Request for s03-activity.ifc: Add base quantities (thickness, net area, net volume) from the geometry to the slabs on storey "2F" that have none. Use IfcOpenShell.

First a look at what the model holds.

```python
import ifcopenshell
import ifcopenshell.util.element
import ifcopenshell.util.unit

model = ifcopenshell.open("s03-activity.ifc")
print(model.schema)
for unit_type in ("LENGTHUNIT", "AREAUNIT", "VOLUMEUNIT"):
    print(unit_type, ifcopenshell.util.unit.calculate_unit_scale(model, unit_type))
storey = next(s for s in model.by_type("IfcBuildingStorey") if s.Name == "2F")
slabs = [e for e in ifcopenshell.util.element.get_decomposition(storey) if e.is_a("IfcSlab")]
for e in sorted(slabs, key=lambda e: e.id()):
    print(e.id(), e.is_a(), e.Name, list(ifcopenshell.util.element.get_psets(e, qtos_only=True)), sep=" | ")
```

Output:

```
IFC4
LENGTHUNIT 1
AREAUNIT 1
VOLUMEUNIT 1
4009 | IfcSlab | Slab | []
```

```python
import ifcopenshell
import ifcopenshell.api.pset
import ifcopenshell.geom
import ifcopenshell.util.element
import ifcopenshell.util.shape
import ifcopenshell.util.unit

model = ifcopenshell.open("s03-activity.ifc")
unit_scale = ifcopenshell.util.unit.calculate_unit_scale(model)
area_scale = ifcopenshell.util.unit.calculate_unit_scale(model, "AREAUNIT")
volume_scale = ifcopenshell.util.unit.calculate_unit_scale(model, "VOLUMEUNIT")
settings = ifcopenshell.geom.settings()

storey = next(s for s in model.by_type("IfcBuildingStorey") if s.Name == "2F")
slabs = [e for e in ifcopenshell.util.element.get_decomposition(storey) if e.is_a("IfcSlab")]

for e in sorted(slabs, key=lambda e: e.id()):
    if ifcopenshell.util.element.get_psets(e, qtos_only=True, should_inherit=False):
        continue
    # Geometry comes back in metres, in the element's own axes.
    shape = ifcopenshell.geom.create_shape(settings, e)
    values = {
        "Width": ifcopenshell.util.shape.get_z(shape.geometry) / unit_scale,
        "NetArea": ifcopenshell.util.shape.get_footprint_area(shape.geometry) / area_scale,
        "NetVolume": ifcopenshell.util.shape.get_volume(shape.geometry) / volume_scale,
    }
    qto = ifcopenshell.api.pset.add_qto(model, product=e, name="Qto_SlabBaseQuantities")
    ifcopenshell.api.pset.edit_qto(model, qto=qto, properties=values)
    print(e.id(), {k: round(v, 3) for k, v in values.items()})

model.write("s03-activity_edited.ifc")
```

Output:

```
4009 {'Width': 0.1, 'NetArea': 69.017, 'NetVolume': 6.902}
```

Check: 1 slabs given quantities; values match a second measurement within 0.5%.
